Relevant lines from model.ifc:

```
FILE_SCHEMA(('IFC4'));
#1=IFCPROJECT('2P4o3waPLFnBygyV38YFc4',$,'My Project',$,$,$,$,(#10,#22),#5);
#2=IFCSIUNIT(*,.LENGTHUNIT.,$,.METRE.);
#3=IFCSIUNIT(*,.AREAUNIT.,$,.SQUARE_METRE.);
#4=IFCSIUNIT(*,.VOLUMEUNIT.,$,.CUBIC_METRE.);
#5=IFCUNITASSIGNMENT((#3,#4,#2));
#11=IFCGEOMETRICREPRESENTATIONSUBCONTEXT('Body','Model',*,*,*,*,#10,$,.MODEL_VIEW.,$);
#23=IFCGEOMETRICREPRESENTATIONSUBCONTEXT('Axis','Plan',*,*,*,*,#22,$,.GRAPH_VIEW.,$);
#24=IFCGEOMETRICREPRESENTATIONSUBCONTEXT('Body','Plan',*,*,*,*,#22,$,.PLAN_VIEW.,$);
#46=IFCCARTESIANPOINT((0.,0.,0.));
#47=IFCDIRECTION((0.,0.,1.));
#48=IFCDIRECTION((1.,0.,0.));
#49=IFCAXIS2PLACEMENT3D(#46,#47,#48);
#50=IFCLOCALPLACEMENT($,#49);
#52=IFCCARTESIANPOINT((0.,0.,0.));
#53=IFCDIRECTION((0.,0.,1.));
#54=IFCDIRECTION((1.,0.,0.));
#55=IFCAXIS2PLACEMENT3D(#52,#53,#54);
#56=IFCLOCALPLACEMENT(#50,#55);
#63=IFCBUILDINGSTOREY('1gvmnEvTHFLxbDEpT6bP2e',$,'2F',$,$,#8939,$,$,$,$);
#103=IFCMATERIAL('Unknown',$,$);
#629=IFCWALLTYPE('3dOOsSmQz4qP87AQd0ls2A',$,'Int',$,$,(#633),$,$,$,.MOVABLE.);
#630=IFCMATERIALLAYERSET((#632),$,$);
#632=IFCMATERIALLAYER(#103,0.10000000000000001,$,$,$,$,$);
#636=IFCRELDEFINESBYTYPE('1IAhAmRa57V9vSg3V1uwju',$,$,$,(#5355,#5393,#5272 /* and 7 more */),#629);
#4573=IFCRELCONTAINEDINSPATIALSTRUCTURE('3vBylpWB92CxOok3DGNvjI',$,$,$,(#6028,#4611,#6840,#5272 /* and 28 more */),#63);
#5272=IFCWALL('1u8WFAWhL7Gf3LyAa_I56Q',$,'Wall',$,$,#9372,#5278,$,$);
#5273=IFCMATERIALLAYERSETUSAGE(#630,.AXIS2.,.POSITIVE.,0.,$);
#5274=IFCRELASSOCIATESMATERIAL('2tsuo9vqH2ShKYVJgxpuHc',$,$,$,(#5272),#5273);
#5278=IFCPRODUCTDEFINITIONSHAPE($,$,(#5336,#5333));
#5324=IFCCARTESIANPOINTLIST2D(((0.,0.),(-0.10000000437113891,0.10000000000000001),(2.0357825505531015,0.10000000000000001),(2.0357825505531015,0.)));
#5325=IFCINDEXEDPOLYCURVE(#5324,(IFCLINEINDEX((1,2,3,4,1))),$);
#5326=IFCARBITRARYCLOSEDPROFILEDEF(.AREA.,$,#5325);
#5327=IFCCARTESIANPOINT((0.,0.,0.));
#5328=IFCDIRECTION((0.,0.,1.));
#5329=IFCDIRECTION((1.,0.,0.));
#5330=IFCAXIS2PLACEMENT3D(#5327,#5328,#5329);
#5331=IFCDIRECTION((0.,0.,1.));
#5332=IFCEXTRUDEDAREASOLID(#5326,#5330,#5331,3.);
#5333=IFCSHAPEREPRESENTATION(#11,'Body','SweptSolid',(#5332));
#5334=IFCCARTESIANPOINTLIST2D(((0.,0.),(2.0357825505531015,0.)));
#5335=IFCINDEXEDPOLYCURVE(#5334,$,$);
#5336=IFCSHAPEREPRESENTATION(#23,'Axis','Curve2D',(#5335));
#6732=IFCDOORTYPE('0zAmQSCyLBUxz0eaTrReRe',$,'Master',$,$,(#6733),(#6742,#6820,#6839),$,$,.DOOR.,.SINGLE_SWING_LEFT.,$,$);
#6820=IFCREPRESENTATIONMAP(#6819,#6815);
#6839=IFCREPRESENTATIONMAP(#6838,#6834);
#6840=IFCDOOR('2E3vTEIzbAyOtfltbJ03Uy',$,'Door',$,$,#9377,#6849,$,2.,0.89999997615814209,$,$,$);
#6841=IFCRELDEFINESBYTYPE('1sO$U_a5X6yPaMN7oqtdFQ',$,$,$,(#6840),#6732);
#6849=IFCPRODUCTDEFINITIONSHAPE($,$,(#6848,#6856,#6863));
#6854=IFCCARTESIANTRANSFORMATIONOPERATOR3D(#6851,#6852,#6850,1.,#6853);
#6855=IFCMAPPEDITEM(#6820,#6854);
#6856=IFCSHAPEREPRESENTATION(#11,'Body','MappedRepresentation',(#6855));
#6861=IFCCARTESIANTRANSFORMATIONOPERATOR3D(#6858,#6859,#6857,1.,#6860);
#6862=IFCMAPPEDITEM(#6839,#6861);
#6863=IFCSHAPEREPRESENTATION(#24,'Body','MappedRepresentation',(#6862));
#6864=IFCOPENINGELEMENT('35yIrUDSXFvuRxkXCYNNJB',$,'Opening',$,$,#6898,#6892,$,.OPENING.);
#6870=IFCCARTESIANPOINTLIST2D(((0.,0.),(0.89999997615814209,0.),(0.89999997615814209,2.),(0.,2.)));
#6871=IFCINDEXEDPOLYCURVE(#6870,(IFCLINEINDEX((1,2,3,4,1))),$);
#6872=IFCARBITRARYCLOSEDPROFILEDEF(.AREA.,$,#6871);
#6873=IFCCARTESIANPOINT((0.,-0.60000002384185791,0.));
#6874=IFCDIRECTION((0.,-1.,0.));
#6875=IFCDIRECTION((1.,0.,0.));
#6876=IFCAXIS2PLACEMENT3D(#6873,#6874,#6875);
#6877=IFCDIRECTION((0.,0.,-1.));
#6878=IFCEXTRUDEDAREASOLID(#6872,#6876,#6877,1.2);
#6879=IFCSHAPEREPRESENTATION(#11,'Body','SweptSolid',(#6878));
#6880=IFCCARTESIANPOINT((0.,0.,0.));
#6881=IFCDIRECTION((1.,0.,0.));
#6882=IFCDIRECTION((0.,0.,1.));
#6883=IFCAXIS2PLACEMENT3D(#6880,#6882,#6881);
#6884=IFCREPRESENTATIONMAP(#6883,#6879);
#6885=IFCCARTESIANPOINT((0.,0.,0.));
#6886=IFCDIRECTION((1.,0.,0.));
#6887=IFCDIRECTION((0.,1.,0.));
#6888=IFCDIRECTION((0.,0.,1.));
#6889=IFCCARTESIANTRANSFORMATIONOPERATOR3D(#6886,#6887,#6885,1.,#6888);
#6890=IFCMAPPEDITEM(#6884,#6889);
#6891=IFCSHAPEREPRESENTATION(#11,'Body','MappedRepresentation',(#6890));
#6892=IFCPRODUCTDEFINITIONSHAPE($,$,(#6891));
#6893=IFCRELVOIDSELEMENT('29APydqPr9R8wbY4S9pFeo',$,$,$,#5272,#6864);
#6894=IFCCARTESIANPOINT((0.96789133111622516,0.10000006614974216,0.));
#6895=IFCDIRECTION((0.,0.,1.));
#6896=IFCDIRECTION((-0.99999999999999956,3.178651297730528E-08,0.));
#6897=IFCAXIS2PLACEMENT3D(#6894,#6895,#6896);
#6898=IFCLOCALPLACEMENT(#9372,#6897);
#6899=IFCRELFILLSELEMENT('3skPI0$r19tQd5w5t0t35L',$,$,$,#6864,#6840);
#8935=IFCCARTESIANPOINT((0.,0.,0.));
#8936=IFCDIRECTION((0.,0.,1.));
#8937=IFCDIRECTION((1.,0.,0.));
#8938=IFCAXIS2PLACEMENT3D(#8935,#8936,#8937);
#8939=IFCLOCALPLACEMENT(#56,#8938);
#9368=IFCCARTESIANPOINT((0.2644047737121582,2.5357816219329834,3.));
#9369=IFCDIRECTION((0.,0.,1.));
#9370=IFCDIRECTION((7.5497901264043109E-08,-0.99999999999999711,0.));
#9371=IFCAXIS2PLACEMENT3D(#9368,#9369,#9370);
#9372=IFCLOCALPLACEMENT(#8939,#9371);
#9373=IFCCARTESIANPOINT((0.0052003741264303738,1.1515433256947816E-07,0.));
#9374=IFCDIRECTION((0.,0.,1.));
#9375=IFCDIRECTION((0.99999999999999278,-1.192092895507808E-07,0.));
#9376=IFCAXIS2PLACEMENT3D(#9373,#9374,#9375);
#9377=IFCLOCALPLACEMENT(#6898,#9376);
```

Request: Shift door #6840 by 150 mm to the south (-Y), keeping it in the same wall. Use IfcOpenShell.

```python
import ifcopenshell
import ifcopenshell.api.geometry
import ifcopenshell.util.placement
import ifcopenshell.util.unit

model = ifcopenshell.open("model.ifc")
unit_scale = ifcopenshell.util.unit.calculate_unit_scale(model)

door = model.by_id(6840)
opening = door.FillsVoids[0].RelatingOpeningElement
wall = opening.VoidsElements[0].RelatingBuildingElement

wall_matrix = ifcopenshell.util.placement.get_local_placement(wall.ObjectPlacement)
shift = wall_matrix[:3, 0] * 0.15 / unit_scale
before = ifcopenshell.util.placement.get_local_placement(door.ObjectPlacement)[:3, 3].copy()

# The door is placed relative to its opening, so it follows when the opening moves.
matrix = ifcopenshell.util.placement.get_local_placement(opening.ObjectPlacement)
matrix[:3, 3] += shift
ifcopenshell.api.geometry.edit_object_placement(
    model, product=opening, matrix=matrix, is_si=False, should_transform_children=True
)

after = ifcopenshell.util.placement.get_local_placement(door.ObjectPlacement)[:3, 3]
print("door moved by", (after - before).round(3) + 0.0)

model.write("model_v2.ifc")
```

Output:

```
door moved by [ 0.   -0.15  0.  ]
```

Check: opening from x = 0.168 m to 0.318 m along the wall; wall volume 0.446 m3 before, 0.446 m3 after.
